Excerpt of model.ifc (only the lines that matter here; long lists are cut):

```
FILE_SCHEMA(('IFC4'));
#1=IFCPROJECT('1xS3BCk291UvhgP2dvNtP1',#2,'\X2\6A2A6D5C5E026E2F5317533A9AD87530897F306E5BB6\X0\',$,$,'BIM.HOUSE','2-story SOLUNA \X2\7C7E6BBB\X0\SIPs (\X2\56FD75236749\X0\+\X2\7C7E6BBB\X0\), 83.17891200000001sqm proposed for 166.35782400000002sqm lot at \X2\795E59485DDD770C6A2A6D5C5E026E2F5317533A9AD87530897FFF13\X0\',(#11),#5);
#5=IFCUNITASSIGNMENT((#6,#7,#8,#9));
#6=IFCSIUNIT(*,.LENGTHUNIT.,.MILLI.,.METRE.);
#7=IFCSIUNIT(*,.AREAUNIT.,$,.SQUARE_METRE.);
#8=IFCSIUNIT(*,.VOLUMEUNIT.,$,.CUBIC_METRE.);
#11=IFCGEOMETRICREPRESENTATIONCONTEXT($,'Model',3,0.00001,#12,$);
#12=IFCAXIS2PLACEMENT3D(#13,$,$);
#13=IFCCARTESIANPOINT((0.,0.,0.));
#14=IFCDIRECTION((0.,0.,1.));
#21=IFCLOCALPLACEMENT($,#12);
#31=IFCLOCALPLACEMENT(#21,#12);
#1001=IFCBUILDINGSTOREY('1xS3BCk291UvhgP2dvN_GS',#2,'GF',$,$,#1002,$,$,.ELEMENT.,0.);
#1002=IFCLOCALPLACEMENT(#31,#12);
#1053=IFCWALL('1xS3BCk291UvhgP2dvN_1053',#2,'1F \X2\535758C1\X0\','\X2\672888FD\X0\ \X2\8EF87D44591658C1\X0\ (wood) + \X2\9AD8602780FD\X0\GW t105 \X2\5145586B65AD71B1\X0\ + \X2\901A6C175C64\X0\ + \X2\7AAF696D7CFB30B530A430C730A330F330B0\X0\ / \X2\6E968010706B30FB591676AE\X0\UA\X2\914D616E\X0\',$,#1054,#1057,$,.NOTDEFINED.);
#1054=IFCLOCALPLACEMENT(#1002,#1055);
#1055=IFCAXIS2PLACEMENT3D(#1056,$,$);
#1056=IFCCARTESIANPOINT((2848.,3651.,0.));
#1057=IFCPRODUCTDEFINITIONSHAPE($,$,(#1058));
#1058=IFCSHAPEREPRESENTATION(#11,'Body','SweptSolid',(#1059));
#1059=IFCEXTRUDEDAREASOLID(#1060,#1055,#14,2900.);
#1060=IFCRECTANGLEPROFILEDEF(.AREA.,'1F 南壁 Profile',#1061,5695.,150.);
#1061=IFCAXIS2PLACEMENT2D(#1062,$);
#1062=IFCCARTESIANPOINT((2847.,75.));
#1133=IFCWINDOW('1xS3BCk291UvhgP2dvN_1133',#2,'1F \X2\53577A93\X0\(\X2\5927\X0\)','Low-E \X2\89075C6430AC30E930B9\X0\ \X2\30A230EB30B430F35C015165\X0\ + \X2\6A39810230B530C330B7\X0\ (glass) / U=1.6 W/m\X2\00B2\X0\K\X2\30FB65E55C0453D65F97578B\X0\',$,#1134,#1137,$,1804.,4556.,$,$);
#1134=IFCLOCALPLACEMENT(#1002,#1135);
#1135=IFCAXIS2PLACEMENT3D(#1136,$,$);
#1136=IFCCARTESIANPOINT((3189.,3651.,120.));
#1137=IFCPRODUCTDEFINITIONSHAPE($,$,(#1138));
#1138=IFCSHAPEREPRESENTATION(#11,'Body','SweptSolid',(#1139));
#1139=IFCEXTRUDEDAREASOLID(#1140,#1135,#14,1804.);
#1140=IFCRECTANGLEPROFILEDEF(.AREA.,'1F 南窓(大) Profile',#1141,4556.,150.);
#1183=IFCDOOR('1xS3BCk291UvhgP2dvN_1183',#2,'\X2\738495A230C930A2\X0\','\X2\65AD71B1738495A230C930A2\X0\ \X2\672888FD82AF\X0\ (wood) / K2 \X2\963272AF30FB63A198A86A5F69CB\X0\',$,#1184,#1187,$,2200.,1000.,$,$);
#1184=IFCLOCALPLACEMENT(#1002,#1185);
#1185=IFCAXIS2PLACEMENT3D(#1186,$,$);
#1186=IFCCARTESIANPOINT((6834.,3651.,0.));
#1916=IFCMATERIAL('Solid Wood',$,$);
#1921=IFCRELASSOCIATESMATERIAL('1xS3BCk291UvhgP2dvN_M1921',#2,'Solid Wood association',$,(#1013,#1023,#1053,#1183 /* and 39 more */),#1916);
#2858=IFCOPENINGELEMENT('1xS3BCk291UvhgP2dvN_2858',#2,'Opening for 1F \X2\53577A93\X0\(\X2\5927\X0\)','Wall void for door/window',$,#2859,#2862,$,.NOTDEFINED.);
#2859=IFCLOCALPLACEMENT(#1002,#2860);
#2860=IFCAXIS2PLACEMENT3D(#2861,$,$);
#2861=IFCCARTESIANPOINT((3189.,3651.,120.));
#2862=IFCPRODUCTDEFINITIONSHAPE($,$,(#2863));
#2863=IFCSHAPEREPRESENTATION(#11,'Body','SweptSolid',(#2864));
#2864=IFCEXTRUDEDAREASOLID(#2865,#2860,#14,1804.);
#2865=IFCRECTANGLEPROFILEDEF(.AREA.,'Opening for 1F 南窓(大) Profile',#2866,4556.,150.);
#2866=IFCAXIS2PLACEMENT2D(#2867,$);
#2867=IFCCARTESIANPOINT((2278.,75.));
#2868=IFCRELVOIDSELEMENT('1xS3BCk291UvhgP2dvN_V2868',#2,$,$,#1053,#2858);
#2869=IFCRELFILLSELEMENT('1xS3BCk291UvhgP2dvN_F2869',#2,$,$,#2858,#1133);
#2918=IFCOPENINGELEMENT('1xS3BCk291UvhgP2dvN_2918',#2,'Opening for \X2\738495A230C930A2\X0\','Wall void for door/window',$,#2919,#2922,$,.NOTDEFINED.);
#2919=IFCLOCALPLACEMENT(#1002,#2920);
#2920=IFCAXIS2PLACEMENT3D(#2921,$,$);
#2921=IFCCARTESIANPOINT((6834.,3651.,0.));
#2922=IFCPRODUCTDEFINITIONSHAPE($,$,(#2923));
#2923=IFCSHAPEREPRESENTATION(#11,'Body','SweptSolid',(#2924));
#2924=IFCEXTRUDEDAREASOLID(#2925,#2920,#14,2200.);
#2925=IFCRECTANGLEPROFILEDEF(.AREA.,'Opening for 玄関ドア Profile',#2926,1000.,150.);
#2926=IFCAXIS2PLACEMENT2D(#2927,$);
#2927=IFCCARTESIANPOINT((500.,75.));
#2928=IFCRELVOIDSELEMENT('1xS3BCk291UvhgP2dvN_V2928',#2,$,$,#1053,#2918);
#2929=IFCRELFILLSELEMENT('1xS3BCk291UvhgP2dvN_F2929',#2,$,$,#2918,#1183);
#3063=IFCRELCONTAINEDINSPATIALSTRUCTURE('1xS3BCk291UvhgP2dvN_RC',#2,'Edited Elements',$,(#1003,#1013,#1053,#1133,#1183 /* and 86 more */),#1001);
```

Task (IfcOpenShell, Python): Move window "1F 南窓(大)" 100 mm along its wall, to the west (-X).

```python
import ifcopenshell
import ifcopenshell.api.geometry
import ifcopenshell.util.placement

model = ifcopenshell.open("model.ifc")

window = model.by_guid("1xS3BCk291UvhgP2dvN_1133")
opening = window.FillsVoids[0].RelatingOpeningElement
wall = opening.VoidsElements[0].RelatingBuildingElement

wall_matrix = ifcopenshell.util.placement.get_local_placement(wall.ObjectPlacement)
shift = wall_matrix[:3, 0] * -100.0
before = ifcopenshell.util.placement.get_local_placement(window.ObjectPlacement)[:3, 3].copy()

# The window is not placed relative to its opening, so move both.
for product in (opening, window):
    matrix = ifcopenshell.util.placement.get_local_placement(product.ObjectPlacement)
    matrix[:3, 3] += shift
    ifcopenshell.api.geometry.edit_object_placement(model, product=product, matrix=matrix, is_si=False)

after = ifcopenshell.util.placement.get_local_placement(window.ObjectPlacement)[:3, 3]
print("window moved by", (after - before).round(3) + 0.0)

model.write("model_edited.ifc")
```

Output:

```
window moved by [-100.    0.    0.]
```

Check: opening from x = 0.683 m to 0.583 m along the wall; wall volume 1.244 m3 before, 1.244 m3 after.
